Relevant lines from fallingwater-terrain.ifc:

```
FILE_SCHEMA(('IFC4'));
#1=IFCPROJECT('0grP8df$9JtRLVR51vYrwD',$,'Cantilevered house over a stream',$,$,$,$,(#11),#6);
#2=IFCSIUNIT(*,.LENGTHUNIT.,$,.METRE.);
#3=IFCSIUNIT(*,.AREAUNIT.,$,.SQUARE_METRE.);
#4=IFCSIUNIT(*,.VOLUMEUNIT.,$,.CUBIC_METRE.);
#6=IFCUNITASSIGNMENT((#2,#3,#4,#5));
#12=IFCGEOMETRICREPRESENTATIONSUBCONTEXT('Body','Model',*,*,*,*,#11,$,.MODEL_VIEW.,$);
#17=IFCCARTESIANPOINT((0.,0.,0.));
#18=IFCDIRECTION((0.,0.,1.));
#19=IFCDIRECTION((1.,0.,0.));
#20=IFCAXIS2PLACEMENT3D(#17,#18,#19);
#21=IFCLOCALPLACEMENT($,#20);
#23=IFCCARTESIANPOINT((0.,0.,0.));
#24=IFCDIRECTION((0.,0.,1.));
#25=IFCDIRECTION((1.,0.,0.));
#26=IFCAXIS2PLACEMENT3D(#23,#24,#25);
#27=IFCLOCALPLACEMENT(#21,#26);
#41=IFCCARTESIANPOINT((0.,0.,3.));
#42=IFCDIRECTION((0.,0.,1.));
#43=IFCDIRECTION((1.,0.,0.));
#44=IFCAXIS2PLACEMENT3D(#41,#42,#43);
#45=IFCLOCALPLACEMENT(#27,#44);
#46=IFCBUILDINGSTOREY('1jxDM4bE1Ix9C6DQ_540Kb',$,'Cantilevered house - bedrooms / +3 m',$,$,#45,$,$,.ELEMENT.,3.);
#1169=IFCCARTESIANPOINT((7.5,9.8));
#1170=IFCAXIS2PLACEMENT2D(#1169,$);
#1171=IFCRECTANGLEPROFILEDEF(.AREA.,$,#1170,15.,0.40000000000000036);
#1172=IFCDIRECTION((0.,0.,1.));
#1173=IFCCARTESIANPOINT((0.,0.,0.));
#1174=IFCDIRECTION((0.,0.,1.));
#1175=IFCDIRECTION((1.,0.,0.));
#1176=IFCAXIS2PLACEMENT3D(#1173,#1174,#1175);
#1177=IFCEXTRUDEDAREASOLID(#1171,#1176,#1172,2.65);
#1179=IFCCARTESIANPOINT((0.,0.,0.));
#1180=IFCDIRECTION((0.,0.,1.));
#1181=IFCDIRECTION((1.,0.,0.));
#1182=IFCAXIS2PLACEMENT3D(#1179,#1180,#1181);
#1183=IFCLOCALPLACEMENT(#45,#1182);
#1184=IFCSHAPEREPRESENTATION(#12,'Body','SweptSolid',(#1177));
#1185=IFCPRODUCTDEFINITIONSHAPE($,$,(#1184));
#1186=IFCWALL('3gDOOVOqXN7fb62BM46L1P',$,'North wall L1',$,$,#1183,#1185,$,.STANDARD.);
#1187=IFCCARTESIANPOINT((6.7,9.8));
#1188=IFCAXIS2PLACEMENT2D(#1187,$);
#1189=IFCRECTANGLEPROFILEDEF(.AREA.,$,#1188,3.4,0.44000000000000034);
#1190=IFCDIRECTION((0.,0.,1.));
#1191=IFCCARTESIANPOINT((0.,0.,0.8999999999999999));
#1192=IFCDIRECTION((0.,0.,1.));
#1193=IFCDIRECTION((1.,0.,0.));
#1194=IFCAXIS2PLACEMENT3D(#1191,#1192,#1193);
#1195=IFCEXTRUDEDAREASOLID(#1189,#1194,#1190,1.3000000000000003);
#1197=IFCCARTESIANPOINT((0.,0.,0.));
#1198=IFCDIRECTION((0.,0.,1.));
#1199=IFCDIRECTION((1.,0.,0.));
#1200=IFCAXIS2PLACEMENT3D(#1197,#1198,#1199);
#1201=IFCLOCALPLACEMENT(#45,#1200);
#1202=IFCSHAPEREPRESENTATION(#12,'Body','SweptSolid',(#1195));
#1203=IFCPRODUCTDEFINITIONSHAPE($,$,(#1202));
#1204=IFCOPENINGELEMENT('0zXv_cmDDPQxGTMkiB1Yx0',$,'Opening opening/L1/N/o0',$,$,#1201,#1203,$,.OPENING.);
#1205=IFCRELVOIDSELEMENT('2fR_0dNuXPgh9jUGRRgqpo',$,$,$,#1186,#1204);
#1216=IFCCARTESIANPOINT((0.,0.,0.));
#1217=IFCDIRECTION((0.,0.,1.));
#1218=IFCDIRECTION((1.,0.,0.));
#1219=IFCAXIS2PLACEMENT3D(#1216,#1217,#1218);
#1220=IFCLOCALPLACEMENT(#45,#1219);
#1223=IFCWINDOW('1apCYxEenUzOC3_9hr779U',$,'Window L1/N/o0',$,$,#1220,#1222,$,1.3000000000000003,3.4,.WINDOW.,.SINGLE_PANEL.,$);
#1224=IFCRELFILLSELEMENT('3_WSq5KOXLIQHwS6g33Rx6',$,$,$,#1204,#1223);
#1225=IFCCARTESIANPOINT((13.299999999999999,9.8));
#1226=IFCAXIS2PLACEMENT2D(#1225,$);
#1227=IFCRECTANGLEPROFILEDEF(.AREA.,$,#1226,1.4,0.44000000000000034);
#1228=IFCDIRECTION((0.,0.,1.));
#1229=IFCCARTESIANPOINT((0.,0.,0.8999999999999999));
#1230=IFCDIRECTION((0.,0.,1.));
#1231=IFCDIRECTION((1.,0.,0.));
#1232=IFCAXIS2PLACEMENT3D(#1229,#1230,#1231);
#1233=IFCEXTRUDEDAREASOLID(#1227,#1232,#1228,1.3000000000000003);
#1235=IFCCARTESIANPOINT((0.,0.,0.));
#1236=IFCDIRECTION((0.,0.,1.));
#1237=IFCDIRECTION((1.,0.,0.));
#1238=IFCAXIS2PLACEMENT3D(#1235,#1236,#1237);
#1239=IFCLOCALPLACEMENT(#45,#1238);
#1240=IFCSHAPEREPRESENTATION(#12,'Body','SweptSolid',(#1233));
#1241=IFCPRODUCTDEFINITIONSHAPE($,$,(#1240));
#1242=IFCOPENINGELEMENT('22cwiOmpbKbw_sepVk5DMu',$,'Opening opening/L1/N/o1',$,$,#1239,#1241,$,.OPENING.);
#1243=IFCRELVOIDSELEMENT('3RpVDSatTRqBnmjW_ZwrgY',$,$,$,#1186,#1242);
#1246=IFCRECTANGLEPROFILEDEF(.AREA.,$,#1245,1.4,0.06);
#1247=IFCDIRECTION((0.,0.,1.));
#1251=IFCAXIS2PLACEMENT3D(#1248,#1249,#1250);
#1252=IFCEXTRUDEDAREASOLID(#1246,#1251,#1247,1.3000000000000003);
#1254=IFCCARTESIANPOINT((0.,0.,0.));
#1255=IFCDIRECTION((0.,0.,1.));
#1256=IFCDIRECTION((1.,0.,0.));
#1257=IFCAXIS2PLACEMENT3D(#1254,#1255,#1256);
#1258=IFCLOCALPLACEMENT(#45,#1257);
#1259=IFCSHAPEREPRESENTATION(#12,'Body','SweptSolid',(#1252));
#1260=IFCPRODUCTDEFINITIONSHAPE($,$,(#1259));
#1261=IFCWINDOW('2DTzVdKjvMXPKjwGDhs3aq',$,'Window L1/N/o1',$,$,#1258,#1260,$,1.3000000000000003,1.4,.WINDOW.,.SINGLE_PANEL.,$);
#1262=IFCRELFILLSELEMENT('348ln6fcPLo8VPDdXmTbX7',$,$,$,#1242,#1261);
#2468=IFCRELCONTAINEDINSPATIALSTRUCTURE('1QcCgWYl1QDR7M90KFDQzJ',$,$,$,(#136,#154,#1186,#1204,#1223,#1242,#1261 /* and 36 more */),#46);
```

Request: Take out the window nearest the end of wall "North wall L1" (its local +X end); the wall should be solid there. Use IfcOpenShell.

```python
import ifcopenshell
import ifcopenshell.api.feature
import ifcopenshell.api.root
import ifcopenshell.geom
import ifcopenshell.util.shape

model = ifcopenshell.open("fallingwater-terrain.ifc")
settings = ifcopenshell.geom.settings()


def volume(element):
    """Net volume in cubic metres, openings subtracted."""
    shape = ifcopenshell.geom.create_shape(settings, element)
    return ifcopenshell.util.shape.get_volume(shape.geometry)


window = model.by_guid("2DTzVdKjvMXPKjwGDhs3aq")
opening = window.FillsVoids[0].RelatingOpeningElement
wall = opening.VoidsElements[0].RelatingBuildingElement
before = volume(wall)

ifcopenshell.api.root.remove_product(model, product=window)
ifcopenshell.api.feature.remove_feature(model, feature=opening)

after = volume(wall)

print(f"wall volume {before:.3f} -> {after:.3f} m3")

model.write("fallingwater-terrain_rev.ifc")
```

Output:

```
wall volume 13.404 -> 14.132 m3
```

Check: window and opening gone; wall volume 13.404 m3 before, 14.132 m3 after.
